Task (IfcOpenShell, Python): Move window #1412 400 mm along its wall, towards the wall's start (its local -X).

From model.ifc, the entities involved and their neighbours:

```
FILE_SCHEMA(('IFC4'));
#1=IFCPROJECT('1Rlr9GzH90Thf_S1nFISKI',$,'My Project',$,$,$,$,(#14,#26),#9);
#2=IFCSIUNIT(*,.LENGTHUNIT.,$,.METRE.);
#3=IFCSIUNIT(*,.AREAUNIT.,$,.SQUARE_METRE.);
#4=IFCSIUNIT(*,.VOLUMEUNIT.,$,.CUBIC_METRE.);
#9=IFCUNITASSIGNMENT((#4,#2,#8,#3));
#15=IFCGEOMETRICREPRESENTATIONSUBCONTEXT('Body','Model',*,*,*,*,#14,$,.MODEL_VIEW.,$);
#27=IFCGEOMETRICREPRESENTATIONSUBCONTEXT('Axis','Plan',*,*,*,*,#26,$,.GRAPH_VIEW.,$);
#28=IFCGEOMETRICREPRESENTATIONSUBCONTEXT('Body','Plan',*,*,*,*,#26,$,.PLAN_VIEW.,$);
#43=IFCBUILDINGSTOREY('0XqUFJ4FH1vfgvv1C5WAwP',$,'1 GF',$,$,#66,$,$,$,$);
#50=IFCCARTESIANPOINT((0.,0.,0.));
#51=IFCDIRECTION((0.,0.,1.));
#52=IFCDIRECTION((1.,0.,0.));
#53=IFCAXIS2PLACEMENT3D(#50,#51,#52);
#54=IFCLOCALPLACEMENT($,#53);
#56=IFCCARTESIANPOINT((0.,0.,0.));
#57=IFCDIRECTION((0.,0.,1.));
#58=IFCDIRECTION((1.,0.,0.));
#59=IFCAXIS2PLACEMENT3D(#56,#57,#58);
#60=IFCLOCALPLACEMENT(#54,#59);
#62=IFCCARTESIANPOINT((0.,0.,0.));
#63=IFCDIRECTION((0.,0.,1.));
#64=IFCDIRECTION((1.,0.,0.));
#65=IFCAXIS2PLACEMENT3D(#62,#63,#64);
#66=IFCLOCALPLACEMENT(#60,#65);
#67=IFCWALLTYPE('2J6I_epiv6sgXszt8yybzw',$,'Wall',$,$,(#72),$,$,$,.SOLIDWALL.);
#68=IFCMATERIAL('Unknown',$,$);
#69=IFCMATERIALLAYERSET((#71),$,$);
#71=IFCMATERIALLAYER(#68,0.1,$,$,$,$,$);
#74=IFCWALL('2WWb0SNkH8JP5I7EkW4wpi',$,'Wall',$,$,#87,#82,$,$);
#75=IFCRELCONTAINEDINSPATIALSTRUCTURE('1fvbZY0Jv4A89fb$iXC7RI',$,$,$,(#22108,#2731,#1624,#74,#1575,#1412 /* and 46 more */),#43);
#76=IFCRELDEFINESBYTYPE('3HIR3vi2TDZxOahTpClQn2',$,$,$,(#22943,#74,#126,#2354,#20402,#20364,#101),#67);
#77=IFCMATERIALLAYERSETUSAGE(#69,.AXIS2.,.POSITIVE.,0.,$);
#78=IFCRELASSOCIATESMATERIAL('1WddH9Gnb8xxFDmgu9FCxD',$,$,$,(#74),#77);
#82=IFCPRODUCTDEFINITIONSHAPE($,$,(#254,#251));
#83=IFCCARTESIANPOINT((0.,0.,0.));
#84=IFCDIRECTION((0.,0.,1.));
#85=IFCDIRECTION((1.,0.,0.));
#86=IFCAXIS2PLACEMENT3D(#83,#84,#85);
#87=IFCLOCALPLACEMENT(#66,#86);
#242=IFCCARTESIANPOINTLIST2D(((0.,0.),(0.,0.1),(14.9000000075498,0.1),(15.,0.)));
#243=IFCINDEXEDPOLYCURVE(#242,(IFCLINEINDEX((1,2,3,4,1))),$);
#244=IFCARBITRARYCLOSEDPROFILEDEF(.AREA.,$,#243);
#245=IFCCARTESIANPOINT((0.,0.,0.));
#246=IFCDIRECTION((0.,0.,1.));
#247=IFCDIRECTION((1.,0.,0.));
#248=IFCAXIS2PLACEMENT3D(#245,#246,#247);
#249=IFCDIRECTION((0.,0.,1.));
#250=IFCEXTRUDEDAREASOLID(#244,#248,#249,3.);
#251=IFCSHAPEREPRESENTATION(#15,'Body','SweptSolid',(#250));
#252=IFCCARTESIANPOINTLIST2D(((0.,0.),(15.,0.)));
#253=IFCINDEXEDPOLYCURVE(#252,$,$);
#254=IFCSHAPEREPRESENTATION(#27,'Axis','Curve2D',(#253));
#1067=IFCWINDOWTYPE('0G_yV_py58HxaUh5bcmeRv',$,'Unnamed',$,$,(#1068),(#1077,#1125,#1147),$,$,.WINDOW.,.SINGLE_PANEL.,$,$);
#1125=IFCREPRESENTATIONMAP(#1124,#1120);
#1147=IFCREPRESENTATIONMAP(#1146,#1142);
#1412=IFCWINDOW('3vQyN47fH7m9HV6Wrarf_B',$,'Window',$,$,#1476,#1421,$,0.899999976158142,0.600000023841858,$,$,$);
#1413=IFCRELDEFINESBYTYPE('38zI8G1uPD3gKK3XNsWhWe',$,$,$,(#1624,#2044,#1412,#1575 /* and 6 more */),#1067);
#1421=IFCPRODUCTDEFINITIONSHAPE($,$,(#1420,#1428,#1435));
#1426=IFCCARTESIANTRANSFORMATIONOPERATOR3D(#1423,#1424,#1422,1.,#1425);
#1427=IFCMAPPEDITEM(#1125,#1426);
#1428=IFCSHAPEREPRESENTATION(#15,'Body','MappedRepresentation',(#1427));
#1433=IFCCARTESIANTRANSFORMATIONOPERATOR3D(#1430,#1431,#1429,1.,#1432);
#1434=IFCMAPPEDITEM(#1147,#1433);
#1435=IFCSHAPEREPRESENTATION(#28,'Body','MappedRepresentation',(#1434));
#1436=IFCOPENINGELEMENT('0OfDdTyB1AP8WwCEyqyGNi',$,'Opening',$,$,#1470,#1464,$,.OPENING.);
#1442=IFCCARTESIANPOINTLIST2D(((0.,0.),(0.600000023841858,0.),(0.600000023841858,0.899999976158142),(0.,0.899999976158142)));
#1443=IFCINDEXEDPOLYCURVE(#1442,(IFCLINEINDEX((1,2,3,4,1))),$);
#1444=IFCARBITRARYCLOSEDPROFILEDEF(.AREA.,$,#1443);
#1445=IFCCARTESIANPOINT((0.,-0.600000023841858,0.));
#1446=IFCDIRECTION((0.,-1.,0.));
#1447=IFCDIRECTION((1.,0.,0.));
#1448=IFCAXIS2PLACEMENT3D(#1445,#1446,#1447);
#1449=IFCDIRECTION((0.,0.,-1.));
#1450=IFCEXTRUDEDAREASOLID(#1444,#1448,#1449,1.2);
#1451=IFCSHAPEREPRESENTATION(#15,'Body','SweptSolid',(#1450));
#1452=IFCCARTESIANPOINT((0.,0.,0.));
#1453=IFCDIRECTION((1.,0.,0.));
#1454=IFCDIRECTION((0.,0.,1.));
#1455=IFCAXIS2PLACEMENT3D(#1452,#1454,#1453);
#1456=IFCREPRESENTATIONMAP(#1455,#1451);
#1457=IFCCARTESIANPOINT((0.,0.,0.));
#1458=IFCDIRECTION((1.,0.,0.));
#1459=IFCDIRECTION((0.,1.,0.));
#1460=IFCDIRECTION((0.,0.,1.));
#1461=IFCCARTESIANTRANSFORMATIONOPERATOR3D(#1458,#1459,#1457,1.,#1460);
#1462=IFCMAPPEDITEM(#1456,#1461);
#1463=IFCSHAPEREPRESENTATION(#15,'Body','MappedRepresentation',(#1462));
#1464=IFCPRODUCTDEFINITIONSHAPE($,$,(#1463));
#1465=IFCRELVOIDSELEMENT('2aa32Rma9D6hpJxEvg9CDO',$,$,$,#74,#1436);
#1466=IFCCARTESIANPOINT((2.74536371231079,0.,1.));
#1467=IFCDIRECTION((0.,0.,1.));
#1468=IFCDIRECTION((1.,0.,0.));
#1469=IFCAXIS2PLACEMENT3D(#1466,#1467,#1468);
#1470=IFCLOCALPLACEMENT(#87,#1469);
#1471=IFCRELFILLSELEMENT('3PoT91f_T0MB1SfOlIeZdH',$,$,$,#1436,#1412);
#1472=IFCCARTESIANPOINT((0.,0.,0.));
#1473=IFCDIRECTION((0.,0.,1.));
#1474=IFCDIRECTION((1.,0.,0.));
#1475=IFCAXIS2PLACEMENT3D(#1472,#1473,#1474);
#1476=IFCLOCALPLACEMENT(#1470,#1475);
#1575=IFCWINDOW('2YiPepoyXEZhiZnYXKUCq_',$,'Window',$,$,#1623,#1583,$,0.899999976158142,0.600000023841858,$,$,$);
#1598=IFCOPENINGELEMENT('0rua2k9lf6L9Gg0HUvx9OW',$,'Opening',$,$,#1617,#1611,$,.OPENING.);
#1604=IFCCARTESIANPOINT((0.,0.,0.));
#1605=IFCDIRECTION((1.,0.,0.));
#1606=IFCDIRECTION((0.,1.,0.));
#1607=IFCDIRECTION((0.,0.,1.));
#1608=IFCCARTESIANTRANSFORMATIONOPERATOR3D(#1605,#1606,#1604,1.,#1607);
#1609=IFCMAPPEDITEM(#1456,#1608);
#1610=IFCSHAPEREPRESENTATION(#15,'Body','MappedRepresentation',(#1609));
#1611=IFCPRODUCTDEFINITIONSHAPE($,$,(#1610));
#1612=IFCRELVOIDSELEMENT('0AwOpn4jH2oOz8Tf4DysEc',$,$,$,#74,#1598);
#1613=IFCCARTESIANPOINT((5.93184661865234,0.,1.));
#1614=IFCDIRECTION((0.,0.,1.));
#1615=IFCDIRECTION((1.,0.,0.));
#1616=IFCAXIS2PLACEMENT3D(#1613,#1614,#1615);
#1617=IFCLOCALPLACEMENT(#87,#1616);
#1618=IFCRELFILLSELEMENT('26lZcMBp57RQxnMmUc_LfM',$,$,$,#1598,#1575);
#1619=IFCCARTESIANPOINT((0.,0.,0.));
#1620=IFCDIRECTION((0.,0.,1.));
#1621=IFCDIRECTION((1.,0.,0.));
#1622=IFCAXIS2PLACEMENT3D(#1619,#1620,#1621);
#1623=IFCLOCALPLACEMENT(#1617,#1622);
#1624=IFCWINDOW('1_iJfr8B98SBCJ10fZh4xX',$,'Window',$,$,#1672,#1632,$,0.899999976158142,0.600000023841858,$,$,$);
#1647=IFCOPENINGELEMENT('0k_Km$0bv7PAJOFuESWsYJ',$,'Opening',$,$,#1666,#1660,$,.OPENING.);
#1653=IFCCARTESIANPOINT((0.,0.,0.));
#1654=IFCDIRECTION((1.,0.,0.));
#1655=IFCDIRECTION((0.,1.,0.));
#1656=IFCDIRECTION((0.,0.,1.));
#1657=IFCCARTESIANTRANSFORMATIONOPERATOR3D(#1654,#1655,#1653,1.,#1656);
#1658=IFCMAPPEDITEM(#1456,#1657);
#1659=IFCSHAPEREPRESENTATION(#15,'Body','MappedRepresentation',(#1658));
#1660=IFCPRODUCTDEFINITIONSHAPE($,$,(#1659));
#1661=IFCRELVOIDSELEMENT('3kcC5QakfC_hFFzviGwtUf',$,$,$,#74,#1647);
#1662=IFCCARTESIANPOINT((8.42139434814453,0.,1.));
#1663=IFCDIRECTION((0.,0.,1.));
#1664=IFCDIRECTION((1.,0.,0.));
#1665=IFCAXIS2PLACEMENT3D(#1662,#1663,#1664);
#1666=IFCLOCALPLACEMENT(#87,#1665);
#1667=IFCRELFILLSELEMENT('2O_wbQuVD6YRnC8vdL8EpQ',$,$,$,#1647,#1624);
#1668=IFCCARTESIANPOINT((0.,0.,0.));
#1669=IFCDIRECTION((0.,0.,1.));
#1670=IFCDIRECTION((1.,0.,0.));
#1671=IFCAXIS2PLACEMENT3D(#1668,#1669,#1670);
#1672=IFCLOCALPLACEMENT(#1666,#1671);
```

```python
import ifcopenshell
import ifcopenshell.api.geometry
import ifcopenshell.util.placement

model = ifcopenshell.open("model.ifc")

window = model.by_guid("3vQyN47fH7m9HV6Wrarf_B")
opening = window.FillsVoids[0].RelatingOpeningElement
wall = opening.VoidsElements[0].RelatingBuildingElement

wall_matrix = ifcopenshell.util.placement.get_local_placement(wall.ObjectPlacement)
shift = wall_matrix[:3, 0] * -0.4
before = ifcopenshell.util.placement.get_local_placement(window.ObjectPlacement)[:3, 3].copy()

# The window is placed relative to its opening, so it follows when the opening moves.
matrix = ifcopenshell.util.placement.get_local_placement(opening.ObjectPlacement)
matrix[:3, 3] += shift
ifcopenshell.api.geometry.edit_object_placement(
    model, product=opening, matrix=matrix, is_si=False, should_transform_children=True
)

after = ifcopenshell.util.placement.get_local_placement(window.ObjectPlacement)[:3, 3]
print("window moved by", (after - before).round(3) + 0.0)

model.write("model_edited.ifc")
```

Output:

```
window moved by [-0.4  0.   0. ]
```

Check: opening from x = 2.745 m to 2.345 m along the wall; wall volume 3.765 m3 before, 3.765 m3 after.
